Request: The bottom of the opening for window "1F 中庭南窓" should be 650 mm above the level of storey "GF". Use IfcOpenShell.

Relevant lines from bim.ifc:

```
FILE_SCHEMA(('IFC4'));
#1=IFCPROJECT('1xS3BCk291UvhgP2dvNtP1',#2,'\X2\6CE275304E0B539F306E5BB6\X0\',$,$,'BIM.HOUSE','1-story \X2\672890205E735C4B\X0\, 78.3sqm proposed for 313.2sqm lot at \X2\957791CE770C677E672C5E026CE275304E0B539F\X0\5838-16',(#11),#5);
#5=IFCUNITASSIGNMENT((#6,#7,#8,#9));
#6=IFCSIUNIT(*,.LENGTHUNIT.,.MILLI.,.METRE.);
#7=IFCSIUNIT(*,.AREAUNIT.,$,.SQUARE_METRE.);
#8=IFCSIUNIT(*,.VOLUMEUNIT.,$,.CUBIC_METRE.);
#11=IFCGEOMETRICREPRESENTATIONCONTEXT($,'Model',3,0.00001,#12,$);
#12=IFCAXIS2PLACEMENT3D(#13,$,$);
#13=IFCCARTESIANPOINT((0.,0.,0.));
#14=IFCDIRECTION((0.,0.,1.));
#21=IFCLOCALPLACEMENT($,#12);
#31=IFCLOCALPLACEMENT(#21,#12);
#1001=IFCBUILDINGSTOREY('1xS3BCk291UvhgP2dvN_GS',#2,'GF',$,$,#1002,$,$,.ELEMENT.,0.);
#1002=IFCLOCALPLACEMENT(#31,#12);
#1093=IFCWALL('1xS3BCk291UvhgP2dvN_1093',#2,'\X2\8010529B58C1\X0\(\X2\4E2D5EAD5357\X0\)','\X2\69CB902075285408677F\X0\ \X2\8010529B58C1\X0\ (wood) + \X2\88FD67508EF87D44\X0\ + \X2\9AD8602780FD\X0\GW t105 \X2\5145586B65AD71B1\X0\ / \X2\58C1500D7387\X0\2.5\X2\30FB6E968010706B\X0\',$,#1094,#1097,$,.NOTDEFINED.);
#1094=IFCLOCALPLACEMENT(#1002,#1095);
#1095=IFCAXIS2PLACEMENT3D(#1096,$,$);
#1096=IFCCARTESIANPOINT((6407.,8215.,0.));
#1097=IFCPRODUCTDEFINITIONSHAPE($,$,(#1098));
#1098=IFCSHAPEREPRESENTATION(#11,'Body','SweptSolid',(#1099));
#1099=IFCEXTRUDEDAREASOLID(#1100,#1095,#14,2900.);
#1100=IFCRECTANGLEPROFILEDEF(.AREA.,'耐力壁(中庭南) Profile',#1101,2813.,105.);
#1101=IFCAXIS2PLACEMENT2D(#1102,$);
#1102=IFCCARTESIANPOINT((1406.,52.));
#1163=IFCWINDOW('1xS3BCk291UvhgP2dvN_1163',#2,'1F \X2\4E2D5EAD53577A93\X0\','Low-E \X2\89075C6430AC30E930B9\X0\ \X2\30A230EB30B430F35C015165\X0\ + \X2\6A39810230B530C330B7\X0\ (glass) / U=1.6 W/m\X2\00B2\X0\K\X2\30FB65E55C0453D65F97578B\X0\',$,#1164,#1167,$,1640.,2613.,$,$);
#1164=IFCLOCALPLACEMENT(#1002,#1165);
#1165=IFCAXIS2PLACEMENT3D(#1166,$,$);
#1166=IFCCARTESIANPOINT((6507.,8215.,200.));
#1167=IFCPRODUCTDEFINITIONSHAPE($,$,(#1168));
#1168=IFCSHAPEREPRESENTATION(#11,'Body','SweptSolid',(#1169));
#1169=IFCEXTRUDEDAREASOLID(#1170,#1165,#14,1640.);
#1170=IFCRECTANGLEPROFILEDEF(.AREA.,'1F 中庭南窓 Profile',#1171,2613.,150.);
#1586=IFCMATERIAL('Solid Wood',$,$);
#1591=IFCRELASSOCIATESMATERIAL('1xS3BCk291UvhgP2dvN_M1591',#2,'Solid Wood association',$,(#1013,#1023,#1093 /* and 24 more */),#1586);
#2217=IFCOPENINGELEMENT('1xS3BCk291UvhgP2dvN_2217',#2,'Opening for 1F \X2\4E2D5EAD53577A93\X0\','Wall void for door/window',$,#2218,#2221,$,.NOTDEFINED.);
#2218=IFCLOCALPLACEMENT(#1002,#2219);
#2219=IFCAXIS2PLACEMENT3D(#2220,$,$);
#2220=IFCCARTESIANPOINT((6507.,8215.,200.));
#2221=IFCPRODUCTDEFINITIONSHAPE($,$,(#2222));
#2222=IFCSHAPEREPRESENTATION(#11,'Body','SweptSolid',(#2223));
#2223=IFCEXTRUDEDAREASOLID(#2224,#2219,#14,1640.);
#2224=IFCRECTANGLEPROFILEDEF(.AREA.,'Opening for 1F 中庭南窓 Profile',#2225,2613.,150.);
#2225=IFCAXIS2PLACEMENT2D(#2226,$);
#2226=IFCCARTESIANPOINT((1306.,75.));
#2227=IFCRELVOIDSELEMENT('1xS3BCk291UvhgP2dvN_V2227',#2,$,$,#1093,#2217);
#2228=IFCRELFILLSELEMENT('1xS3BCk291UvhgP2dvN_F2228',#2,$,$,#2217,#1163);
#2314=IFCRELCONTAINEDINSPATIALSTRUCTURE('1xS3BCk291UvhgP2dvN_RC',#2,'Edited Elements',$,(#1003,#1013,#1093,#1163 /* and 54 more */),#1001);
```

```python
import numpy as np
import ifcopenshell
import ifcopenshell.api.geometry
import ifcopenshell.geom
import ifcopenshell.util.element
import ifcopenshell.util.placement
import ifcopenshell.util.shape
import ifcopenshell.util.unit

model = ifcopenshell.open("bim.ifc")
unit_scale = ifcopenshell.util.unit.calculate_unit_scale(model)

window = model.by_id(1163)
opening = window.FillsVoids[0].RelatingOpeningElement
storey = ifcopenshell.util.element.get_container(window, ifc_class="IfcBuildingStorey")
level = ifcopenshell.util.placement.get_local_placement(storey.ObjectPlacement)[2, 3]

# The opening's origin need not be at the sill, so measure its lowest point.
shape = ifcopenshell.geom.create_shape(ifcopenshell.geom.settings(), opening)
bottom = ifcopenshell.util.shape.get_shape_bottom_elevation(shape, shape.geometry) / unit_scale
dz = level + 0.65 / unit_scale - bottom

shift = np.array([0.0, 0.0, dz])
# The window is not placed relative to its opening, so move both.
for product in (opening, window):
    matrix = ifcopenshell.util.placement.get_local_placement(product.ObjectPlacement)
    matrix[:3, 3] += shift
    ifcopenshell.api.geometry.edit_object_placement(model, product=product, matrix=matrix, is_si=False)

print(f"moved by {dz * unit_scale:+.3f} m")

model.write("bim_updated.ifc")
```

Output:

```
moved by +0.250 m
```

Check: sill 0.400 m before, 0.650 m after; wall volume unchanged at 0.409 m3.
